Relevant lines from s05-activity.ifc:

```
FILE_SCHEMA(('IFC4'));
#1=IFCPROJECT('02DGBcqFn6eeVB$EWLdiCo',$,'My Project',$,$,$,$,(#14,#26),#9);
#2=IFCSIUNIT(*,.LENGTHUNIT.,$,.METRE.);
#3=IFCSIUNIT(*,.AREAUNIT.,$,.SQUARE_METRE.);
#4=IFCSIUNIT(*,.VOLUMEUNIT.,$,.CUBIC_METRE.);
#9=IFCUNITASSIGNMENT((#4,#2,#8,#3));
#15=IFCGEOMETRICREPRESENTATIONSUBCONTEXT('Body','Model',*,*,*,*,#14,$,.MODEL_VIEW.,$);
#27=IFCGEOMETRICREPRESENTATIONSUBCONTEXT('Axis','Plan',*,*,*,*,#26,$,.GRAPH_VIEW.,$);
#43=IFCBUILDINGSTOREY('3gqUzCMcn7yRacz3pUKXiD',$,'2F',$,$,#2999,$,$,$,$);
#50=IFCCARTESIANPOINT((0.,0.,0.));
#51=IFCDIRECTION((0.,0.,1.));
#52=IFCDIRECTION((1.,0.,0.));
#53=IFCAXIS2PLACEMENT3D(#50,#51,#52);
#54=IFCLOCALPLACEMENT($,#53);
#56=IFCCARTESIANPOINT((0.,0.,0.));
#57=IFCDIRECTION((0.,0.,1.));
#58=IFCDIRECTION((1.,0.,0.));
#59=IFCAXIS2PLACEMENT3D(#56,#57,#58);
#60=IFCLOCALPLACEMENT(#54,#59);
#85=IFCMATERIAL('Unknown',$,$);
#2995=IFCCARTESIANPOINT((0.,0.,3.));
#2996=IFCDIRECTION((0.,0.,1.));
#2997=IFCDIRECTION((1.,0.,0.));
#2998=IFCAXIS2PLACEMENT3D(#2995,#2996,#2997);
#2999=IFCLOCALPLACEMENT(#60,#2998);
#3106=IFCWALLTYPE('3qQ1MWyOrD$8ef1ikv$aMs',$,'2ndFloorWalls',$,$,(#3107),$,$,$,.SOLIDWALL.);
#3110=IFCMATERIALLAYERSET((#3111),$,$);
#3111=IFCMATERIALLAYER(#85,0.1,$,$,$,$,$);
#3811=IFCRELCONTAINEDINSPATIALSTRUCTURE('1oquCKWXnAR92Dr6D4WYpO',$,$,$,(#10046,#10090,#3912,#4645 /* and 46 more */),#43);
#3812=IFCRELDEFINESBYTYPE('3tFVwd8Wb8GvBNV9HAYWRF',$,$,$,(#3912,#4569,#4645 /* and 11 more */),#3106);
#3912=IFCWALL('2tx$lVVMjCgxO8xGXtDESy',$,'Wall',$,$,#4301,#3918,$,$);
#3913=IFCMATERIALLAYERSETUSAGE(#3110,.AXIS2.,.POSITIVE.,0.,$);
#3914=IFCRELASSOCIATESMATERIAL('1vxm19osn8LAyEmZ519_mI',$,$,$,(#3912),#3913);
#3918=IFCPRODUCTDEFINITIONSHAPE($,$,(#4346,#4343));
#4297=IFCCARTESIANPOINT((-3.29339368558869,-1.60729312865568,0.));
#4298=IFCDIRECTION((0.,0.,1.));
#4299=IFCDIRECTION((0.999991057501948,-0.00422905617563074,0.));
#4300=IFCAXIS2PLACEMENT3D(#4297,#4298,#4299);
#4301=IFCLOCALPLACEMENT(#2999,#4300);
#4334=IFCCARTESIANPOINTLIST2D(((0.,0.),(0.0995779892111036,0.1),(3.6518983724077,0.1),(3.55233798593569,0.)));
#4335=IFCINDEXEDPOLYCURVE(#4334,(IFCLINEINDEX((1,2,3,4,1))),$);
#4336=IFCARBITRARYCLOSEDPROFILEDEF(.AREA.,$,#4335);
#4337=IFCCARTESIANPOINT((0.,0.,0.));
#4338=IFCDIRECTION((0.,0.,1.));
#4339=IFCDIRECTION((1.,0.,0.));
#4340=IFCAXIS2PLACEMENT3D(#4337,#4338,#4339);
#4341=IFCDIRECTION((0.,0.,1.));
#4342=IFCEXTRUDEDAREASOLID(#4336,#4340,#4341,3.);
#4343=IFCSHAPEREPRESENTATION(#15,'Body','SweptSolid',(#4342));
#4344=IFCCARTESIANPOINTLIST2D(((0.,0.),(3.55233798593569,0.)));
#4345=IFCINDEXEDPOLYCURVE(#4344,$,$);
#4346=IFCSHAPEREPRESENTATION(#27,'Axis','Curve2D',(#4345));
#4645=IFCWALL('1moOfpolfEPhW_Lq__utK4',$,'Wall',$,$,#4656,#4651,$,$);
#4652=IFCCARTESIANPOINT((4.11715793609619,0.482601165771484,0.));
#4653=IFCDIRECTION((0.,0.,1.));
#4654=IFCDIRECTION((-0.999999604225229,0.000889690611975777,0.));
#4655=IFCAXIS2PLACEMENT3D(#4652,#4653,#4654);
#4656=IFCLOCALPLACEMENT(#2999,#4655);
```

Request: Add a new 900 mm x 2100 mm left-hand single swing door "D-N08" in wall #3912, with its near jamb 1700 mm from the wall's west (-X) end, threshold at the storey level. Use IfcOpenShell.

```python
import numpy as np
import ifcopenshell
import ifcopenshell.api.feature
import ifcopenshell.api.geometry
import ifcopenshell.api.root
import ifcopenshell.api.spatial
import ifcopenshell.geom
import ifcopenshell.util.element
import ifcopenshell.util.placement
import ifcopenshell.util.representation
import ifcopenshell.util.shape
import ifcopenshell.util.unit

model = ifcopenshell.open("s05-activity.ifc")
unit_scale = ifcopenshell.util.unit.calculate_unit_scale(model)
settings = ifcopenshell.geom.settings()


def volume(element):
    """Net volume in cubic metres, openings subtracted."""
    shape = ifcopenshell.geom.create_shape(settings, element)
    return ifcopenshell.util.shape.get_volume(shape.geometry)


wall = model.by_id(3912)
storey = ifcopenshell.util.element.get_container(wall, ifc_class="IfcBuildingStorey")
context = ifcopenshell.util.representation.get_context(model, "Model", "Body", "MODEL_VIEW")
before = volume(wall)

width, height, from_end, sill = 0.9, 2.1, 1.7, 0.0  # metres

# The wall runs along its own X axis, and the end named is its -X end.
wall_shape = ifcopenshell.geom.create_shape(settings, wall)
x, y, z = ifcopenshell.util.shape.get_vertices(wall_shape.geometry).T
start = x.min() + from_end
face, thickness = float(y.min()), float(y.max() - y.min())
wall_matrix = ifcopenshell.util.placement.get_local_placement(wall.ObjectPlacement)
level = ifcopenshell.util.placement.get_local_placement(storey.ObjectPlacement)[2, 3]


def in_wall(x, y):
    """Placement at x, y metres in the wall's axes, at sill height."""
    matrix = wall_matrix.copy()
    matrix[:, 3] = wall_matrix @ np.array([x / unit_scale, y / unit_scale, 0.0, 1.0])
    matrix[2, 3] = level + sill / unit_scale
    return matrix


# Opening: a box that overshoots both wall faces by 50 mm.
opening = ifcopenshell.api.root.create_entity(model, ifc_class="IfcOpeningElement", predefined_type="OPENING")
box = ifcopenshell.api.geometry.add_wall_representation(
    model, context=context, length=width, height=height, thickness=thickness + 0.1
)
ifcopenshell.api.geometry.assign_representation(model, product=opening, representation=box)
ifcopenshell.api.geometry.edit_object_placement(model, product=opening, matrix=in_wall(start, face - 0.05), is_si=False)
ifcopenshell.api.feature.add_feature(model, feature=opening, element=wall)

door = ifcopenshell.api.root.create_entity(model, ifc_class="IfcDoor", name="D-N08", predefined_type="DOOR")
door.OverallWidth, door.OverallHeight = width / unit_scale, height / unit_scale
door.OperationType = "SINGLE_SWING_LEFT"
body = ifcopenshell.api.geometry.add_door_representation(
    model,
    context=context,
    overall_width=door.OverallWidth,
    overall_height=door.OverallHeight,
    operation_type="SINGLE_SWING_LEFT",
    lining_properties={"LiningDepth": thickness / unit_scale, "ThresholdDepth": thickness / unit_scale},
)
ifcopenshell.api.geometry.assign_representation(model, product=door, representation=body)
ifcopenshell.api.spatial.assign_container(model, products=[door], relating_structure=storey)
ifcopenshell.api.feature.add_filling(model, opening=opening, element=door)

# The lining spans the wall, so the door starts at the wall face.
ifcopenshell.api.geometry.edit_object_placement(model, product=door, matrix=in_wall(start, face), is_si=False)

after = volume(wall)

print(f"wall volume {before:.3f} -> {after:.3f} m3")

model.write("s05-activity_updated.ifc")
```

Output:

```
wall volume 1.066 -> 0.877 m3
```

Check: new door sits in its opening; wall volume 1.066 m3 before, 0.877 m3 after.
